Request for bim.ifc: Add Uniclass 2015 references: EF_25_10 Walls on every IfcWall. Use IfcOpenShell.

First a look at what the model holds.

```python
import ifcopenshell

model = ifcopenshell.open("bim.ifc")
print(model.schema)
print("classifications:", [c.Name for c in model.by_type("IfcClassification")])
for ifc_class in ("IfcDoor", "IfcRoof", "IfcStair", "IfcWall", "IfcWindow"):
    print(ifc_class, len(model.by_type(ifc_class)))
```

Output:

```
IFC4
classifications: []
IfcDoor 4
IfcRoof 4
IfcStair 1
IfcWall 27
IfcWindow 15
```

```python
import ifcopenshell
import ifcopenshell.api.classification

model = ifcopenshell.open("bim.ifc")

system = ifcopenshell.api.classification.add_classification(model, classification="Uniclass 2015")

codes = {
    "IfcWall": ("EF_25_10", "Walls"),
}
for ifc_class, (code, name) in codes.items():
    products = model.by_type(ifc_class)
    ifcopenshell.api.classification.add_reference(
        model, products=products, classification=system, identification=code, name=name
    )
    print(code, len(products))

model.write("bim_updated.ifc")
```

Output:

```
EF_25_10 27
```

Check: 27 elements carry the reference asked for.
